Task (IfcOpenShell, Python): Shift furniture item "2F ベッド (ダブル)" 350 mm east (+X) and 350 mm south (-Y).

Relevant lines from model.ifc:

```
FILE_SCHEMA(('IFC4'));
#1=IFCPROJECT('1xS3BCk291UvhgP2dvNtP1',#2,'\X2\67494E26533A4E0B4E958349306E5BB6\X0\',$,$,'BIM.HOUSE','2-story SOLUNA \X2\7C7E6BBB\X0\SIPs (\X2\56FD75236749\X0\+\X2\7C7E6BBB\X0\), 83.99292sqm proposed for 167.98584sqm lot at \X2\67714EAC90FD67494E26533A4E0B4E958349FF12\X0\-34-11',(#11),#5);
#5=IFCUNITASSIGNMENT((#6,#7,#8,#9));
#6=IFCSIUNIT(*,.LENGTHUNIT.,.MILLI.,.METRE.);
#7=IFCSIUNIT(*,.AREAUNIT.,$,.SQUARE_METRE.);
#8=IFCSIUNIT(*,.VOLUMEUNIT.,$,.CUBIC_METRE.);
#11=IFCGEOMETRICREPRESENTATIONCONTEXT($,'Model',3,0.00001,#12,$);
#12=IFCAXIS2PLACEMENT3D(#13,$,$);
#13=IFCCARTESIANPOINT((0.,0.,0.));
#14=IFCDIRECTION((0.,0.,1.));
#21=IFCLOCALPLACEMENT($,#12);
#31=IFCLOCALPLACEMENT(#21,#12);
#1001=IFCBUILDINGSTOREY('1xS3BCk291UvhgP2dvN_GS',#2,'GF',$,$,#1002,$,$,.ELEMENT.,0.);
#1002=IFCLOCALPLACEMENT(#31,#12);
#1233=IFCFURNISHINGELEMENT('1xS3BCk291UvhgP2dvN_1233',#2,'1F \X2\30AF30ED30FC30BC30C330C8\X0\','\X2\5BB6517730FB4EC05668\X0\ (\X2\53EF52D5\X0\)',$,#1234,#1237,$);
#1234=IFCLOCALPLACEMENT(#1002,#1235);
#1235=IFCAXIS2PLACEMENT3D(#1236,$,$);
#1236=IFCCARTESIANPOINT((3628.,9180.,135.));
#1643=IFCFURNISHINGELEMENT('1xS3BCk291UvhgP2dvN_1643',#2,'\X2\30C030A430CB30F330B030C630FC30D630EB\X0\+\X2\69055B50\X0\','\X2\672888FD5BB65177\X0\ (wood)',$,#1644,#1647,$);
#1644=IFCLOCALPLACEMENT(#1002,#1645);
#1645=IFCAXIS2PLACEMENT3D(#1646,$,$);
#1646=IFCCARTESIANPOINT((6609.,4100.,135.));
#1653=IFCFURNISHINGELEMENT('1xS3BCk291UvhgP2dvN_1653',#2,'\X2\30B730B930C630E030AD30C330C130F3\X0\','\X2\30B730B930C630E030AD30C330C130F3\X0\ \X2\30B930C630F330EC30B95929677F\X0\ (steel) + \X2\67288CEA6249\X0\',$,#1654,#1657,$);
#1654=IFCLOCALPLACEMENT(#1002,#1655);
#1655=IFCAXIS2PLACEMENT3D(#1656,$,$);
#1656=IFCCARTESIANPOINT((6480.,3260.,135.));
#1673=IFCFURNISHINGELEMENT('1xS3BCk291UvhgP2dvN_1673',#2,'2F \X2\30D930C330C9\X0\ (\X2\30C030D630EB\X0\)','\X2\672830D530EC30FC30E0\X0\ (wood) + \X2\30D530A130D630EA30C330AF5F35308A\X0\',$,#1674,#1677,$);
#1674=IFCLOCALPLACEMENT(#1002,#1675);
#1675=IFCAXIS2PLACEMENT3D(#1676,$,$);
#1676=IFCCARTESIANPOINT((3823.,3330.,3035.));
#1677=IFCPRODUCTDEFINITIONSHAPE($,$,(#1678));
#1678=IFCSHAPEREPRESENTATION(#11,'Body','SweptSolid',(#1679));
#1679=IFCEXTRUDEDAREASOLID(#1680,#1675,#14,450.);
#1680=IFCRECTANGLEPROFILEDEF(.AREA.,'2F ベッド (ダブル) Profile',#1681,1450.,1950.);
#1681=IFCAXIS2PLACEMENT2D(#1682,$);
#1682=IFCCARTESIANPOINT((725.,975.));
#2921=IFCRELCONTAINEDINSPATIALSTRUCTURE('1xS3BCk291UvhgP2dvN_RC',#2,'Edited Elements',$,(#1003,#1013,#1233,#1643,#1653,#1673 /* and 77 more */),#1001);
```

```python
import ifcopenshell
import ifcopenshell.api.geometry
import ifcopenshell.util.placement

model = ifcopenshell.open("model.ifc")

item = model.by_guid("1xS3BCk291UvhgP2dvN_1673")
matrix = ifcopenshell.util.placement.get_local_placement(item.ObjectPlacement)
matrix[0, 3] += 350.0
matrix[1, 3] -= 350.0
ifcopenshell.api.geometry.edit_object_placement(model, product=item, matrix=matrix, is_si=False)

print(ifcopenshell.util.placement.get_local_placement(item.ObjectPlacement).round(3) + 0.0)

model.write("model_edited.ifc")
```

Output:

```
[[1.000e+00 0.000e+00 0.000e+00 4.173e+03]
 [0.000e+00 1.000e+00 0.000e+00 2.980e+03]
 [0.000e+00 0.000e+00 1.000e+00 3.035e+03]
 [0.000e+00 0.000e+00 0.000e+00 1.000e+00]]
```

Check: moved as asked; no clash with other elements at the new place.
